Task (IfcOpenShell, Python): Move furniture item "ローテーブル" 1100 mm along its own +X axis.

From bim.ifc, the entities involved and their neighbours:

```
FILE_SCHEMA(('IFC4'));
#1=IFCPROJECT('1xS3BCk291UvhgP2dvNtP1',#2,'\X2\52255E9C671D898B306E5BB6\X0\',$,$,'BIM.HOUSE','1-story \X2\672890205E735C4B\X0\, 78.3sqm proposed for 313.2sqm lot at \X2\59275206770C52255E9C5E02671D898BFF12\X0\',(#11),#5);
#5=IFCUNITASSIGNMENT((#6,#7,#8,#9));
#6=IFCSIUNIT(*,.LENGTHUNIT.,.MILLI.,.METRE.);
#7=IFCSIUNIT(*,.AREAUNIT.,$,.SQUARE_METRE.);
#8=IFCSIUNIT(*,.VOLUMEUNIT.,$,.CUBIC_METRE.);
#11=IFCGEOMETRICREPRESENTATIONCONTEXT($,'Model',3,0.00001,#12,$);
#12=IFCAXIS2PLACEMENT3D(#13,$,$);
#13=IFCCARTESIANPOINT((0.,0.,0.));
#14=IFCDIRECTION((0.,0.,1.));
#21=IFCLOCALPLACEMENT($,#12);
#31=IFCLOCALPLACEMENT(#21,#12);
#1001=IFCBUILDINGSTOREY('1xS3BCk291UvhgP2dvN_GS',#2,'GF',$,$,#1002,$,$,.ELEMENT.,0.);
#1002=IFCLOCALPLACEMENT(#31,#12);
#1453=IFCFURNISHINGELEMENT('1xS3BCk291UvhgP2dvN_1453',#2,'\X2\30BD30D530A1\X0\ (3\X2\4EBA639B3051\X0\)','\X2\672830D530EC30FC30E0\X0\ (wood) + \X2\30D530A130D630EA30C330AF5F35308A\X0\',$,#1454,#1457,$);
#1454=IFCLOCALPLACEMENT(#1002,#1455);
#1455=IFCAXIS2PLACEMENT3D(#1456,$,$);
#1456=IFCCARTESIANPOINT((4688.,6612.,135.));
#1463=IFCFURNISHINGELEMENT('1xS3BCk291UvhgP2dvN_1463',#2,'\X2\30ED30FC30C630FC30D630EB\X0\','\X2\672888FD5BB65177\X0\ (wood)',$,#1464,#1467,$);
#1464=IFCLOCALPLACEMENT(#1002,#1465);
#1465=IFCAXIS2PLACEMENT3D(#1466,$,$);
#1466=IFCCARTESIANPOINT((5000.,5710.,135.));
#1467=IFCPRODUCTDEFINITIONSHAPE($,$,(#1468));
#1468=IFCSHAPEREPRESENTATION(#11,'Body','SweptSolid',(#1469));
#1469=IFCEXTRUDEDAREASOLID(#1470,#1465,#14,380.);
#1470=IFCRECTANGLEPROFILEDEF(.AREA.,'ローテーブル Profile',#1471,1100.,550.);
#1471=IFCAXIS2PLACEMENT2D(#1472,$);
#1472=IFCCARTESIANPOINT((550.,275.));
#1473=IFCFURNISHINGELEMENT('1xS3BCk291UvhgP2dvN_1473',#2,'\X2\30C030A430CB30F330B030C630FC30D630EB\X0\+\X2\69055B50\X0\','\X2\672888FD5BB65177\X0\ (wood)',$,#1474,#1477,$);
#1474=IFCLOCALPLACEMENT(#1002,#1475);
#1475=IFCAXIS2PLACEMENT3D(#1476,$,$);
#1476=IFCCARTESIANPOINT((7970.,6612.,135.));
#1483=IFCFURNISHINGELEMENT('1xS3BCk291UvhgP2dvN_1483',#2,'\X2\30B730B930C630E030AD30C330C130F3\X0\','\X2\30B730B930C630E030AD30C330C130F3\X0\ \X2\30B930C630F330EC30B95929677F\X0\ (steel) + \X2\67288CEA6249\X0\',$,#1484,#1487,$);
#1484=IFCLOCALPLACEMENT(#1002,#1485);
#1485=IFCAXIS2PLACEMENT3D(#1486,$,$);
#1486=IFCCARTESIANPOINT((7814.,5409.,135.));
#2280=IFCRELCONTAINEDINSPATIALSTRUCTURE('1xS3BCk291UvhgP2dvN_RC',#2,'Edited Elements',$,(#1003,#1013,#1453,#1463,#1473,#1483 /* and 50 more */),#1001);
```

```python
import ifcopenshell
import ifcopenshell.api.geometry
import ifcopenshell.util.placement
import ifcopenshell.util.unit

model = ifcopenshell.open("bim.ifc")
unit_scale = ifcopenshell.util.unit.calculate_unit_scale(model)

item = model.by_guid("1xS3BCk291UvhgP2dvN_1463")
matrix = ifcopenshell.util.placement.get_local_placement(item.ObjectPlacement)
matrix[:3, 3] += matrix[:3, 0] * 1.1 / unit_scale
ifcopenshell.api.geometry.edit_object_placement(model, product=item, matrix=matrix, is_si=False)

print(ifcopenshell.util.placement.get_local_placement(item.ObjectPlacement).round(3) + 0.0)

model.write("bim-out.ifc")
```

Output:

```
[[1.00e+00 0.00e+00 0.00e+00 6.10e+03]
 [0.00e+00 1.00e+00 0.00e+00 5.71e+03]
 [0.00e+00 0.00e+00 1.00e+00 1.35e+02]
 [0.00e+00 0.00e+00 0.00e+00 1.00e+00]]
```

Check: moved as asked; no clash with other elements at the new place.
